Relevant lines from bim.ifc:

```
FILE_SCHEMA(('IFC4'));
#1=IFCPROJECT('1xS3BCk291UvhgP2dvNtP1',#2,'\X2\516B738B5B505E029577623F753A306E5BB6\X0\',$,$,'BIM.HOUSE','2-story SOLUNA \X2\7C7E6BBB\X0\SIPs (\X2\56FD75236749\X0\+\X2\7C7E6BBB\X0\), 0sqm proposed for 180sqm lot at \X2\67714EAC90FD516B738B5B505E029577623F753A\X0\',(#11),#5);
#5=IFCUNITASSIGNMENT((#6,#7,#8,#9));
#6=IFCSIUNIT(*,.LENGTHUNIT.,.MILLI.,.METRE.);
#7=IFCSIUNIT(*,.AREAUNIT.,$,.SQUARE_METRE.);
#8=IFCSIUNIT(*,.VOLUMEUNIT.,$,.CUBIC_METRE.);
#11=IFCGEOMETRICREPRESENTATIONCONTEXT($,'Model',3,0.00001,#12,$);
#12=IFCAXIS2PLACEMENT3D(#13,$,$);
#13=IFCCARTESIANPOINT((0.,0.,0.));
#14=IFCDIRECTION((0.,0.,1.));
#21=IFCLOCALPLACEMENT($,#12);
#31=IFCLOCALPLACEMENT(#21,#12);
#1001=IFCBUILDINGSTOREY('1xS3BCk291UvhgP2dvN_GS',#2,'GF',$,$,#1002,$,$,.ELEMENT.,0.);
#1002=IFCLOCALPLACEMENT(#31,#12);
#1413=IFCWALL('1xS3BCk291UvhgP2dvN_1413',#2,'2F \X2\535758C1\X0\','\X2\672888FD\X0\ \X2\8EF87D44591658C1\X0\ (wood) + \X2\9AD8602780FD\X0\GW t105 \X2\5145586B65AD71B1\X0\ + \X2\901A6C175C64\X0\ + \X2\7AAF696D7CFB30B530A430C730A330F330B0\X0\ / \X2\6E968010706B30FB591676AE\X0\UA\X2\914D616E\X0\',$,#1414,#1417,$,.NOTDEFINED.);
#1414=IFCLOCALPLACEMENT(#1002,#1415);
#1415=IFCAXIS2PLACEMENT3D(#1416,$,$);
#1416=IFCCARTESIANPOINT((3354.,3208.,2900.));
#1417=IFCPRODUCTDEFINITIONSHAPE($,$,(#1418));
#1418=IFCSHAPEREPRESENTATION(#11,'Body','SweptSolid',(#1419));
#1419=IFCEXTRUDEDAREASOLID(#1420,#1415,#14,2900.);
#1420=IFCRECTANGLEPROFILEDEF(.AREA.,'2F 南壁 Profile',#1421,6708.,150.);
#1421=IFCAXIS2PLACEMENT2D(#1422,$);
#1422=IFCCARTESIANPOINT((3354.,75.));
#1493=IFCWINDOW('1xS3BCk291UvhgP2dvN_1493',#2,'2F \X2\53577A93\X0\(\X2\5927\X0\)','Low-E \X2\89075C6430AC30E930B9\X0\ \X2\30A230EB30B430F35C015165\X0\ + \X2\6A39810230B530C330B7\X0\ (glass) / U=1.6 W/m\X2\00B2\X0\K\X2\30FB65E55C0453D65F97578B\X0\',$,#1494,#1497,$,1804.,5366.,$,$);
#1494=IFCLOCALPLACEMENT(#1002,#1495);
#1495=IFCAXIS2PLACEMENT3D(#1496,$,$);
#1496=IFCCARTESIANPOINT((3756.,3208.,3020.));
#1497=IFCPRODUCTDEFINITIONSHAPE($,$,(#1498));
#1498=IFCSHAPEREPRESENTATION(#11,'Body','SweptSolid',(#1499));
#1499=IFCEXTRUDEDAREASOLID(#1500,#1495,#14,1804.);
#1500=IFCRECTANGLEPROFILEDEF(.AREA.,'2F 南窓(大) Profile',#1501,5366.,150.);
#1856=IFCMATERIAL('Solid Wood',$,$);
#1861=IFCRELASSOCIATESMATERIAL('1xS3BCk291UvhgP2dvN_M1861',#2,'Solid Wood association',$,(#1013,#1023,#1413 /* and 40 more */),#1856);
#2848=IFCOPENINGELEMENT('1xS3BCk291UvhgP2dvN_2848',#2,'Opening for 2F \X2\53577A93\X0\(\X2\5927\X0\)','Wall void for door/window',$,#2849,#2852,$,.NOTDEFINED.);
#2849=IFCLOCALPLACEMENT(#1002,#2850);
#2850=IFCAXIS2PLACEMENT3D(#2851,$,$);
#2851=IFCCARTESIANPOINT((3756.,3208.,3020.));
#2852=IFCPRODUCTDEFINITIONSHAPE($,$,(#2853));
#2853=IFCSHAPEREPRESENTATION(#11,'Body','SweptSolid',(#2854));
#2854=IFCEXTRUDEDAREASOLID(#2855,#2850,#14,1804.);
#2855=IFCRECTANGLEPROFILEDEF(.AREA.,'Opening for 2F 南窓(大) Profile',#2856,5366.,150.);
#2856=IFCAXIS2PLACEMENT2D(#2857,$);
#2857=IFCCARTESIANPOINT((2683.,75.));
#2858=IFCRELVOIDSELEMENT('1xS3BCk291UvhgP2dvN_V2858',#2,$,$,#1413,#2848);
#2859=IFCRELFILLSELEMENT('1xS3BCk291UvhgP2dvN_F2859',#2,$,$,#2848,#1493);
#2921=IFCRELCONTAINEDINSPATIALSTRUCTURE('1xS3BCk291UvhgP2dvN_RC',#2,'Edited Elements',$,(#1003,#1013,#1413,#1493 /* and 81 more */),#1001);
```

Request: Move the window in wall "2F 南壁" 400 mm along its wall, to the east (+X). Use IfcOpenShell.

```python
import ifcopenshell
import ifcopenshell.api.geometry
import ifcopenshell.util.placement
import ifcopenshell.util.unit

model = ifcopenshell.open("bim.ifc")
unit_scale = ifcopenshell.util.unit.calculate_unit_scale(model)

window = model.by_guid("1xS3BCk291UvhgP2dvN_1493")
opening = window.FillsVoids[0].RelatingOpeningElement
wall = opening.VoidsElements[0].RelatingBuildingElement

wall_matrix = ifcopenshell.util.placement.get_local_placement(wall.ObjectPlacement)
shift = wall_matrix[:3, 0] * 0.4 / unit_scale
before = ifcopenshell.util.placement.get_local_placement(window.ObjectPlacement)[:3, 3].copy()

# The window is not placed relative to its opening, so move both.
for product in (opening, window):
    matrix = ifcopenshell.util.placement.get_local_placement(product.ObjectPlacement)
    matrix[:3, 3] += shift
    ifcopenshell.api.geometry.edit_object_placement(model, product=product, matrix=matrix, is_si=False)

after = ifcopenshell.util.placement.get_local_placement(window.ObjectPlacement)[:3, 3]
print("window moved by", (after - before).round(3) + 0.0)

model.write("bim_edited.ifc")
```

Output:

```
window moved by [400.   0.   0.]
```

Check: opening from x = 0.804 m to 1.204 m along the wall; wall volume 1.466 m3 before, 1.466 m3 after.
